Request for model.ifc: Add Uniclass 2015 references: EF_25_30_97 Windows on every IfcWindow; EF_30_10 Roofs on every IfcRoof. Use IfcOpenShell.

First a look at what the model holds.

```python
import ifcopenshell

model = ifcopenshell.open("model.ifc")
print(model.schema)
print("classifications:", [c.Name for c in model.by_type("IfcClassification")])
for ifc_class in ("IfcDoor", "IfcRoof", "IfcStair", "IfcWall", "IfcWindow"):
    print(ifc_class, len(model.by_type(ifc_class)))
```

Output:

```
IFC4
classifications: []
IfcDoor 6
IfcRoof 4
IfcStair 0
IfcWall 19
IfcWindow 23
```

```python
import ifcopenshell
import ifcopenshell.api.classification

model = ifcopenshell.open("model.ifc")

system = ifcopenshell.api.classification.add_classification(model, classification="Uniclass 2015")

codes = {
    "IfcWindow": ("EF_25_30_97", "Windows"),
    "IfcRoof": ("EF_30_10", "Roofs"),
}
for ifc_class, (code, name) in codes.items():
    products = model.by_type(ifc_class)
    ifcopenshell.api.classification.add_reference(
        model, products=products, classification=system, identification=code, name=name
    )
    print(code, len(products))

model.write("model_rev.ifc")
```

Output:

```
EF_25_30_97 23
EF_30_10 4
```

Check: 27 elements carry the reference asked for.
